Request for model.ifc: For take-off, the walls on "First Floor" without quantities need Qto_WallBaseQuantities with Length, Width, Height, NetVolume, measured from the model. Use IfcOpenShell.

First a look at what the model holds.

```python
import ifcopenshell
import ifcopenshell.util.element
import ifcopenshell.util.unit

model = ifcopenshell.open("model.ifc")
print(model.schema)
for unit_type in ("LENGTHUNIT", "AREAUNIT", "VOLUMEUNIT"):
    print(unit_type, ifcopenshell.util.unit.calculate_unit_scale(model, unit_type))
storey = next(s for s in model.by_type("IfcBuildingStorey") if s.Name == "First Floor")
walls = [e for e in ifcopenshell.util.element.get_decomposition(storey) if e.is_a("IfcWall")]
for e in sorted(walls, key=lambda e: e.id()):
    print(e.id(), e.is_a(), e.Name, list(ifcopenshell.util.element.get_psets(e, qtos_only=True)), sep=" | ")
```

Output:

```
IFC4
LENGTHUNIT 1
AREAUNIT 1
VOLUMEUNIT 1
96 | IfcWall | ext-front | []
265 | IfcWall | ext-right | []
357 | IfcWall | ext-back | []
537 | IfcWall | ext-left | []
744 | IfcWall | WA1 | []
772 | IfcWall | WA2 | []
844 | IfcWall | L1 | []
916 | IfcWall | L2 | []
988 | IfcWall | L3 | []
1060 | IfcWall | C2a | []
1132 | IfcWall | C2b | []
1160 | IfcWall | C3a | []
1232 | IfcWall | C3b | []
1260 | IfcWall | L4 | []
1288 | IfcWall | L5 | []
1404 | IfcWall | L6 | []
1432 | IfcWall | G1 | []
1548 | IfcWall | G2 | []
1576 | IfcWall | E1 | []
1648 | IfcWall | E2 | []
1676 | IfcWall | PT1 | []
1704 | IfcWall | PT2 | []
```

```python
import ifcopenshell
import ifcopenshell.api.pset
import ifcopenshell.geom
import ifcopenshell.util.element
import ifcopenshell.util.shape
import ifcopenshell.util.unit

model = ifcopenshell.open("model.ifc")
unit_scale = ifcopenshell.util.unit.calculate_unit_scale(model)
volume_scale = ifcopenshell.util.unit.calculate_unit_scale(model, "VOLUMEUNIT")
settings = ifcopenshell.geom.settings()

storey = next(s for s in model.by_type("IfcBuildingStorey") if s.Name == "First Floor")
walls = [e for e in ifcopenshell.util.element.get_decomposition(storey) if e.is_a("IfcWall")]

for e in sorted(walls, key=lambda e: e.id()):
    if ifcopenshell.util.element.get_psets(e, qtos_only=True, should_inherit=False):
        continue
    # Geometry comes back in metres, in the element's own axes.
    shape = ifcopenshell.geom.create_shape(settings, e)
    values = {
        "Length": ifcopenshell.util.shape.get_x(shape.geometry) / unit_scale,
        "Width": ifcopenshell.util.shape.get_y(shape.geometry) / unit_scale,
        "Height": ifcopenshell.util.shape.get_z(shape.geometry) / unit_scale,
        "NetVolume": ifcopenshell.util.shape.get_volume(shape.geometry) / volume_scale,
    }
    qto = ifcopenshell.api.pset.add_qto(model, product=e, name="Qto_WallBaseQuantities")
    ifcopenshell.api.pset.edit_qto(model, qto=qto, properties=values)
    print(e.id(), {k: round(v, 3) for k, v in values.items()})

model.write("model_updated.ifc")
```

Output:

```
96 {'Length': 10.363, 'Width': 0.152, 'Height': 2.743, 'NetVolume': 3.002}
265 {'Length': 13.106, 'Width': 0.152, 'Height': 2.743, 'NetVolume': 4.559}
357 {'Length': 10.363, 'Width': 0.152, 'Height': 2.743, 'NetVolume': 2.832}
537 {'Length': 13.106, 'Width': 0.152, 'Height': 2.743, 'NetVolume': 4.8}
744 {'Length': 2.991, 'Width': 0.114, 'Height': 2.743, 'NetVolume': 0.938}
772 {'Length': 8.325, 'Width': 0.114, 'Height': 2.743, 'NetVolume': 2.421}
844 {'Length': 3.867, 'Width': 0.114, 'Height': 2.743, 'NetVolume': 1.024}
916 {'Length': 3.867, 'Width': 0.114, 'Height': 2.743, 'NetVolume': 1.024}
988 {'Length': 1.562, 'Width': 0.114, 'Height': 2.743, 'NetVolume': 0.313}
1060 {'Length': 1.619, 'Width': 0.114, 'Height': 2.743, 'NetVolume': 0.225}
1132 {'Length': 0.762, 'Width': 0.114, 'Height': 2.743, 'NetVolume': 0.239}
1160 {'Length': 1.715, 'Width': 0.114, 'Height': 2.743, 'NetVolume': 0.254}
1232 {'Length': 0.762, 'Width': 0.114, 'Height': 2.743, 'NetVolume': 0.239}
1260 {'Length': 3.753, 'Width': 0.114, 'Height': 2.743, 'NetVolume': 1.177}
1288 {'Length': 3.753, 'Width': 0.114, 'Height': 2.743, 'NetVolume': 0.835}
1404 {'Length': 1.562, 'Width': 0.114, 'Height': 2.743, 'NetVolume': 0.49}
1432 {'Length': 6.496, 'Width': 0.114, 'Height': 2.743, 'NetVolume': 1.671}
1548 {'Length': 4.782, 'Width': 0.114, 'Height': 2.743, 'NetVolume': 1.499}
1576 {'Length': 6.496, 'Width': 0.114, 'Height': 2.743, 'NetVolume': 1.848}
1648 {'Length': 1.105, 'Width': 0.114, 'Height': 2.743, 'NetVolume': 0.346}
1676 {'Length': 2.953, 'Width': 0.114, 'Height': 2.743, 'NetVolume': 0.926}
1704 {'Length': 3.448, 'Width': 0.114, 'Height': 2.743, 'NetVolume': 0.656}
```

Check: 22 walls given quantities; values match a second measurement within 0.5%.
